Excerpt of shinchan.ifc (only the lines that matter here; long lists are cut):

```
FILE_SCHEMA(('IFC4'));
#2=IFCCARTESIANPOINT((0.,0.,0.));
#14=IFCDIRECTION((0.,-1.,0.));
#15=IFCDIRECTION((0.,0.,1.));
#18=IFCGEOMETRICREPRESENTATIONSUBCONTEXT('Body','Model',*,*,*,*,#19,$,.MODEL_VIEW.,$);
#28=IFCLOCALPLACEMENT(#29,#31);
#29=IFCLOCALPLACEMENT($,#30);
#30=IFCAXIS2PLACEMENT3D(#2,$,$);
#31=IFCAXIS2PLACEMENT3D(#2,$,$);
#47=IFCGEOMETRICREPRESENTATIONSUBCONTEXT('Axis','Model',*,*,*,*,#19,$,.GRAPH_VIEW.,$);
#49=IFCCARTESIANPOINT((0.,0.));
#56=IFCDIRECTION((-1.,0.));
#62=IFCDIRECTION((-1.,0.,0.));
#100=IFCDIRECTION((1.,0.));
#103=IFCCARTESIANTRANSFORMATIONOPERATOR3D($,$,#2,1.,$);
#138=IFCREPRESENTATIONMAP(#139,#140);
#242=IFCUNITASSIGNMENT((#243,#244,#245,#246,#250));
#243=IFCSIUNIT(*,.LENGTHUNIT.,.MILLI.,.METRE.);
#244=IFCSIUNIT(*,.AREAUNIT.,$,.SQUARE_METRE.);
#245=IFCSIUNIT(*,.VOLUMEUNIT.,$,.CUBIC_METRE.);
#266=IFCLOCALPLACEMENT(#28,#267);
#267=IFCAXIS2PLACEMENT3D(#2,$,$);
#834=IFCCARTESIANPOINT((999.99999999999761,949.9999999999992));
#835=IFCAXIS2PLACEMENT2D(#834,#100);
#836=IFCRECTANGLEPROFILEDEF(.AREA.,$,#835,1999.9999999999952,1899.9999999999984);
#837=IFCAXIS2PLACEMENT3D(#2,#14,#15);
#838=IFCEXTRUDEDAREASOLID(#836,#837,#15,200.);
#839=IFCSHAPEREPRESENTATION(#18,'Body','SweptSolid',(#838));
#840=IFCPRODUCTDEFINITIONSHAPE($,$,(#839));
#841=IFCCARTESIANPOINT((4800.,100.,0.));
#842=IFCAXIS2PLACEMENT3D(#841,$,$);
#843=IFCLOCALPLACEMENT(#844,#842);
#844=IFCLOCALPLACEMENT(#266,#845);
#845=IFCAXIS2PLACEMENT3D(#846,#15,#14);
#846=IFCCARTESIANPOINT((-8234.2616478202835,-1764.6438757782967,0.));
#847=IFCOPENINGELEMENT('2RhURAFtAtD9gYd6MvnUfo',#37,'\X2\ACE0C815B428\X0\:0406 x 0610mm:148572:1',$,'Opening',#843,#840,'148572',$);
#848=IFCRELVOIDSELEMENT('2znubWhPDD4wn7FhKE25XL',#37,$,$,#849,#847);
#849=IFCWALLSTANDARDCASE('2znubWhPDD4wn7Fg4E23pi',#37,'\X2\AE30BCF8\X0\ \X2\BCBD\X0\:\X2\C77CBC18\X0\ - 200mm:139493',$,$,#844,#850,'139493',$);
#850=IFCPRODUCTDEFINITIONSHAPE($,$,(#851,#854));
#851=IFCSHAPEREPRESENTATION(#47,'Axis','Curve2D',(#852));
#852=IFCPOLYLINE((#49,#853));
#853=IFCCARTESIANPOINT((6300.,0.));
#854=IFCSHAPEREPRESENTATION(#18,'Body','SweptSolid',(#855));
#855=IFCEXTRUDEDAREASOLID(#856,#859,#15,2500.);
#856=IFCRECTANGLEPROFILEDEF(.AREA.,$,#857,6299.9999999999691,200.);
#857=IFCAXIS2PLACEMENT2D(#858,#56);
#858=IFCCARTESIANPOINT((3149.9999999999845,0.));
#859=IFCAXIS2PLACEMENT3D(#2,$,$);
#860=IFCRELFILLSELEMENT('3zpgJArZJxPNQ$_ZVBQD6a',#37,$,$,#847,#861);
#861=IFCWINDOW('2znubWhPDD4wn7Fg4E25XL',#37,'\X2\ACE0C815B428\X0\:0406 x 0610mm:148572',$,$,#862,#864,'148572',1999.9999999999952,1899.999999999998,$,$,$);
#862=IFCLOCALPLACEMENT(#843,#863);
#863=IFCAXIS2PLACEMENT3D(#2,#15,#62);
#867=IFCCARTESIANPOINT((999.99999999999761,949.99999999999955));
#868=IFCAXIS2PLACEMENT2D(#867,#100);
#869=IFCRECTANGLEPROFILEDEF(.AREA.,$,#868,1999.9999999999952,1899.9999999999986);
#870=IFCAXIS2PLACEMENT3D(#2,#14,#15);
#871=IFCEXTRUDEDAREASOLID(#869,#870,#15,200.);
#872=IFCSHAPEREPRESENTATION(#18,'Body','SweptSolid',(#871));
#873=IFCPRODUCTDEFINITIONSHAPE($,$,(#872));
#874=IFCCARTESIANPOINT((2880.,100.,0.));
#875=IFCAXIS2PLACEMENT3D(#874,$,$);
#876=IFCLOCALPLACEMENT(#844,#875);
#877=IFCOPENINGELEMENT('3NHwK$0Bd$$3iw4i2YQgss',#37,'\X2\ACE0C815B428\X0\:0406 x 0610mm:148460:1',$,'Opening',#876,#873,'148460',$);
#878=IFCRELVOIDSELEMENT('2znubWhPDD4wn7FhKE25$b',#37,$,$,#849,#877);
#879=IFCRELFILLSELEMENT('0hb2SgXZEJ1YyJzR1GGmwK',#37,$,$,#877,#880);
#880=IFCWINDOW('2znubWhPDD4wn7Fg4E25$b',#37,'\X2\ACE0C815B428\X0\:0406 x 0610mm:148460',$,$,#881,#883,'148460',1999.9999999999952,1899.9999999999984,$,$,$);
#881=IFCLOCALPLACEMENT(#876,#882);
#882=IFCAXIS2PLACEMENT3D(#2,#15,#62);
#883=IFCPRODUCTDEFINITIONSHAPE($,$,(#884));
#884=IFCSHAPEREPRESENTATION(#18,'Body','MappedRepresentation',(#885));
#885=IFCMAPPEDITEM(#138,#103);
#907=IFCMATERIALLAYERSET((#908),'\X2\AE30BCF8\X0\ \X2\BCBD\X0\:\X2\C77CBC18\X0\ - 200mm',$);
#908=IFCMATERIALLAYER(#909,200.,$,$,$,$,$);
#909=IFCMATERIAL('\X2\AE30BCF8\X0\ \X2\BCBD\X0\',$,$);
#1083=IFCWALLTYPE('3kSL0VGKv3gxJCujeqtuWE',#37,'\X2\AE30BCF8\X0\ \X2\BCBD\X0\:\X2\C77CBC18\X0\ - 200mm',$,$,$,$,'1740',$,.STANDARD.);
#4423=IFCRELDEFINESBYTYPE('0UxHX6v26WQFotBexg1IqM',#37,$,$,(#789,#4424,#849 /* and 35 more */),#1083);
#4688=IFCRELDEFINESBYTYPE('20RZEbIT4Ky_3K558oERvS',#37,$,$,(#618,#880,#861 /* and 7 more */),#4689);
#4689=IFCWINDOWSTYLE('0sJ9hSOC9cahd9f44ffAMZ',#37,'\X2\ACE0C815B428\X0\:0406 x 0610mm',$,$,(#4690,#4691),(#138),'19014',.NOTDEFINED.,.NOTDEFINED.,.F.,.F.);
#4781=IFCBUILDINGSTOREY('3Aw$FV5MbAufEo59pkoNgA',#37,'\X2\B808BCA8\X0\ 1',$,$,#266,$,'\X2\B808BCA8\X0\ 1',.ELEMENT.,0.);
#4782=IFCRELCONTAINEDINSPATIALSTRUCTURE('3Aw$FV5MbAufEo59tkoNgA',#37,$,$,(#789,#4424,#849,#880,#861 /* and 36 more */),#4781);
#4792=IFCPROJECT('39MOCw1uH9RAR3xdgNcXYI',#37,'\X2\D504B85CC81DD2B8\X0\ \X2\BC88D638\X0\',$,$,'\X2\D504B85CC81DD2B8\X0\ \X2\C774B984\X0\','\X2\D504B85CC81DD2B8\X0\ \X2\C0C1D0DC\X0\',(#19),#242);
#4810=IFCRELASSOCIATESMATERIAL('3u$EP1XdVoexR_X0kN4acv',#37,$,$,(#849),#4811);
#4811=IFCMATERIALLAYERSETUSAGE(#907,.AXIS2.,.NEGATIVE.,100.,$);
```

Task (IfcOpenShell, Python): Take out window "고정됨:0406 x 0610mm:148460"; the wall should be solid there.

```python
import ifcopenshell
import ifcopenshell.api.feature
import ifcopenshell.api.root
import ifcopenshell.geom
import ifcopenshell.util.shape

model = ifcopenshell.open("shinchan.ifc")
settings = ifcopenshell.geom.settings()


def volume(element):
    """Net volume in cubic metres, openings subtracted."""
    shape = ifcopenshell.geom.create_shape(settings, element)
    return ifcopenshell.util.shape.get_volume(shape.geometry)


window = model.by_guid("2znubWhPDD4wn7Fg4E25$b")
opening = window.FillsVoids[0].RelatingOpeningElement
wall = opening.VoidsElements[0].RelatingBuildingElement
before = volume(wall)

ifcopenshell.api.root.remove_product(model, product=window)
ifcopenshell.api.feature.remove_feature(model, feature=opening)

after = volume(wall)

print(f"wall volume {before:.3f} -> {after:.3f} m3")

model.write("shinchan_edited.ifc")
```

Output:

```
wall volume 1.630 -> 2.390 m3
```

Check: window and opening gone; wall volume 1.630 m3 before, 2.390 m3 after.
